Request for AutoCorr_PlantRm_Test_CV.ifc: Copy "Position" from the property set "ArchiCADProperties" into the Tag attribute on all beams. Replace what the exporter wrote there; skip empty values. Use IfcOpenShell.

First a look at what the model holds.

```python
import ifcopenshell
import ifcopenshell.util.element

model = ifcopenshell.open("AutoCorr_PlantRm_Test_CV.ifc")
print(model.schema)
beams = model.by_type("IfcBeam")
print(len(beams), "beams")
for e in beams[:8]:
    source = ifcopenshell.util.element.get_pset(e, "ArchiCADProperties", "Position")
    target = e.Tag
    print(e.id(), repr(source), repr(target), sep=" | ")
```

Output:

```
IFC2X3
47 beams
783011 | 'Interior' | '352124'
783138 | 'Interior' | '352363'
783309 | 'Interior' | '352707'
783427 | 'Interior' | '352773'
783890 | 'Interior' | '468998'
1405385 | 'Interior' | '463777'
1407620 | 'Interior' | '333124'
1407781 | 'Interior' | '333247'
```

```python
import ifcopenshell
import ifcopenshell.util.element

model = ifcopenshell.open("AutoCorr_PlantRm_Test_CV.ifc")

count = 0
for e in model.by_type("IfcBeam"):
    value = ifcopenshell.util.element.get_pset(e, "ArchiCADProperties", "Position")
    current = e.Tag
    if not value or not value.strip() or current == value:
        continue
    e.Tag = value
    count += 1

print(count, "beams updated")

model.write("AutoCorr_PlantRm_Test_CV_rev.ifc")
```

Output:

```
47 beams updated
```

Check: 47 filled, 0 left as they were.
